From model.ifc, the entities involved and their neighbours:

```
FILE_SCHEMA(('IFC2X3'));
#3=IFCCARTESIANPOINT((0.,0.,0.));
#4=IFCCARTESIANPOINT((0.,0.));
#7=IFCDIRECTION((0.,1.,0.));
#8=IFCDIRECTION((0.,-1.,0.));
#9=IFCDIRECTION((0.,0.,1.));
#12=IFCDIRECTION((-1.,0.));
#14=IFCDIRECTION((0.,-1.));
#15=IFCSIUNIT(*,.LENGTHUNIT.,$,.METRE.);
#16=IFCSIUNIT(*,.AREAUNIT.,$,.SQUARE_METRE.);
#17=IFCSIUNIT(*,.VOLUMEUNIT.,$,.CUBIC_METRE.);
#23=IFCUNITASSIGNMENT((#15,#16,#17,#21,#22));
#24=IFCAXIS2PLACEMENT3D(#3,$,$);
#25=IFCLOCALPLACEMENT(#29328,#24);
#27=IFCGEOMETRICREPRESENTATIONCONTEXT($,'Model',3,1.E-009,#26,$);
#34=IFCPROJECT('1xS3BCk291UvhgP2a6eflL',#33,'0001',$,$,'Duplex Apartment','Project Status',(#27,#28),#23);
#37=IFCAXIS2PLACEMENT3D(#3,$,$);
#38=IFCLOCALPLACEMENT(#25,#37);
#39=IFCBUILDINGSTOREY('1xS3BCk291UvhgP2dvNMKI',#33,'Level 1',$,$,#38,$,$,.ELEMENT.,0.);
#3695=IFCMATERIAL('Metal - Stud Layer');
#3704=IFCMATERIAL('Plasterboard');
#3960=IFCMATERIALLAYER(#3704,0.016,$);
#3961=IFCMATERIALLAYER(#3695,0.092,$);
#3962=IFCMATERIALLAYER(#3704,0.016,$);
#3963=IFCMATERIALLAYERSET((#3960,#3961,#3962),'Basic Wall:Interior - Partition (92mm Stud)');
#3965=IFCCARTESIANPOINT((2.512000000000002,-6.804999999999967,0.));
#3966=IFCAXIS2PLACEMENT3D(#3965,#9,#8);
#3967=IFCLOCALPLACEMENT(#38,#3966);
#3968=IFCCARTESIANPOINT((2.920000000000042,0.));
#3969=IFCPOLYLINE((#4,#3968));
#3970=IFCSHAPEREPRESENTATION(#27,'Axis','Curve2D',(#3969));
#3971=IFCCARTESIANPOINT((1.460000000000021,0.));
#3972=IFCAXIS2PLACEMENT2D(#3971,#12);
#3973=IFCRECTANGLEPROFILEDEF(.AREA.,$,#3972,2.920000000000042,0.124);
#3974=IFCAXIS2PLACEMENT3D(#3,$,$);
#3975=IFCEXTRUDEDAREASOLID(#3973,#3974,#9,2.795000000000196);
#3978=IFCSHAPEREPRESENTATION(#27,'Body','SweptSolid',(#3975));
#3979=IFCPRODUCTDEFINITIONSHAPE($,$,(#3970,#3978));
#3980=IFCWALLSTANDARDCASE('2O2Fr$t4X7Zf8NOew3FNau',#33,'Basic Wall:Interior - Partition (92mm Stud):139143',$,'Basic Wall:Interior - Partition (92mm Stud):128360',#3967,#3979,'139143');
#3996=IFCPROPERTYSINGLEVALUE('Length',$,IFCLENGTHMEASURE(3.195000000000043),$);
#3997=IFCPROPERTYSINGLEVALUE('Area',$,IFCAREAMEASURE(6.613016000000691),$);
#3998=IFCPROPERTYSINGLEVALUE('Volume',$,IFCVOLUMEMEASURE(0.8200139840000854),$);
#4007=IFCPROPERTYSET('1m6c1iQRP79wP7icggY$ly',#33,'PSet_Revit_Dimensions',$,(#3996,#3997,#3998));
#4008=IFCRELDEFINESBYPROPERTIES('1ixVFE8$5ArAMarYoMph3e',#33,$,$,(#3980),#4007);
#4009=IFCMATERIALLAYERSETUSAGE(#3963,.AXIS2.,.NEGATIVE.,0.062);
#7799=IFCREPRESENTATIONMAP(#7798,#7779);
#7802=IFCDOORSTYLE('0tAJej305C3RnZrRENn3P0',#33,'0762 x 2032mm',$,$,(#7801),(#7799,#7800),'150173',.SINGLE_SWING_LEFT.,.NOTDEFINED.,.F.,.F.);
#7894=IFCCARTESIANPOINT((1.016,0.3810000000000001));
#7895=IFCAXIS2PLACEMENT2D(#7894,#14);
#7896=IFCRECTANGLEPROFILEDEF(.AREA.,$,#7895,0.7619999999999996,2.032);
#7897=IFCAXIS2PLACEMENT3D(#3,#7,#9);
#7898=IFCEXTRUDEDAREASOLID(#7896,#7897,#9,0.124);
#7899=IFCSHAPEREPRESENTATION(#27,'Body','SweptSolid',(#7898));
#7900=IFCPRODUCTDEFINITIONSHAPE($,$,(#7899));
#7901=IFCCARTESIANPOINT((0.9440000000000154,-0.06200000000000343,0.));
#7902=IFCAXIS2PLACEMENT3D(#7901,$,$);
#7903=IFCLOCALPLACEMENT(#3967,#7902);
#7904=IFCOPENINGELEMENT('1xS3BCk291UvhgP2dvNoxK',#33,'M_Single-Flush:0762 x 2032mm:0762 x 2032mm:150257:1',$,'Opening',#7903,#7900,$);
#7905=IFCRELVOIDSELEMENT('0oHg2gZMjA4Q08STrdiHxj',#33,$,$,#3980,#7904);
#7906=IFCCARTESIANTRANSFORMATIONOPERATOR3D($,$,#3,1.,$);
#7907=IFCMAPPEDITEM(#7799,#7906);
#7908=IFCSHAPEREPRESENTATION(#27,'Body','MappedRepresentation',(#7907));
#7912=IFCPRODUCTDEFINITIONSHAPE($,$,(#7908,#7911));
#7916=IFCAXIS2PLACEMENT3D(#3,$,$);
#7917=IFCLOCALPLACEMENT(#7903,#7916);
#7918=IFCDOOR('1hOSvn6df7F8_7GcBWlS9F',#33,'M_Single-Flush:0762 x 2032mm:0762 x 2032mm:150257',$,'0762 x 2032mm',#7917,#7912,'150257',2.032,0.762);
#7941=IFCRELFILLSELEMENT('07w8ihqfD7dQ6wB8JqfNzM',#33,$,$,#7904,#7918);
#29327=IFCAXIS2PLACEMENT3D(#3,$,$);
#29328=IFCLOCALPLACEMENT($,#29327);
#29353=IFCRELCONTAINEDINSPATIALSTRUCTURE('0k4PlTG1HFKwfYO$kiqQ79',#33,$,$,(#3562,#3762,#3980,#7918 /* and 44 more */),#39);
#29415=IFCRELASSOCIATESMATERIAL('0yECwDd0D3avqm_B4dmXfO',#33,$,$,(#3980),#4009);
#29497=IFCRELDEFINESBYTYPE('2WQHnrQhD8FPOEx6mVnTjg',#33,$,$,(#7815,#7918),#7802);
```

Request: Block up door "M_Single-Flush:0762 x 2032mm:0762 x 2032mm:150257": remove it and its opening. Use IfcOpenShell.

```python
import ifcopenshell
import ifcopenshell.api.feature
import ifcopenshell.api.pset
import ifcopenshell.api.root
import ifcopenshell.geom
import ifcopenshell.util.element
import ifcopenshell.util.shape
import ifcopenshell.util.unit

model = ifcopenshell.open("model.ifc")
area_scale = ifcopenshell.util.unit.calculate_unit_scale(model, "AREAUNIT")
volume_scale = ifcopenshell.util.unit.calculate_unit_scale(model, "VOLUMEUNIT")
settings = ifcopenshell.geom.settings()


def volume(element):
    """Net volume in cubic metres, openings subtracted."""
    shape = ifcopenshell.geom.create_shape(settings, element)
    return ifcopenshell.util.shape.get_volume(shape.geometry)


door = model.by_id(7918)
opening = door.FillsVoids[0].RelatingOpeningElement
wall = opening.VoidsElements[0].RelatingBuildingElement
before = volume(wall)

ifcopenshell.api.root.remove_product(model, product=door)
ifcopenshell.api.feature.remove_feature(model, feature=opening)

after = volume(wall)
thickness = 0.124  # wall thickness in metres

# Update the wall's stored quantities.
pset = model.by_id(ifcopenshell.util.element.get_pset(wall, "PSet_Revit_Dimensions", should_inherit=False)["id"])
ifcopenshell.api.pset.edit_pset(model, pset=pset, properties={
    "Area": model.create_entity("IfcAreaMeasure", after / thickness / area_scale),
    "Volume": model.create_entity("IfcVolumeMeasure", after / volume_scale),
})

print(f"wall volume {before:.3f} -> {after:.3f} m3")

model.write("model_rev.ifc")
```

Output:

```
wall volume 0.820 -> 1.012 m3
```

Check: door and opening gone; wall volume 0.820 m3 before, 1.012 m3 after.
